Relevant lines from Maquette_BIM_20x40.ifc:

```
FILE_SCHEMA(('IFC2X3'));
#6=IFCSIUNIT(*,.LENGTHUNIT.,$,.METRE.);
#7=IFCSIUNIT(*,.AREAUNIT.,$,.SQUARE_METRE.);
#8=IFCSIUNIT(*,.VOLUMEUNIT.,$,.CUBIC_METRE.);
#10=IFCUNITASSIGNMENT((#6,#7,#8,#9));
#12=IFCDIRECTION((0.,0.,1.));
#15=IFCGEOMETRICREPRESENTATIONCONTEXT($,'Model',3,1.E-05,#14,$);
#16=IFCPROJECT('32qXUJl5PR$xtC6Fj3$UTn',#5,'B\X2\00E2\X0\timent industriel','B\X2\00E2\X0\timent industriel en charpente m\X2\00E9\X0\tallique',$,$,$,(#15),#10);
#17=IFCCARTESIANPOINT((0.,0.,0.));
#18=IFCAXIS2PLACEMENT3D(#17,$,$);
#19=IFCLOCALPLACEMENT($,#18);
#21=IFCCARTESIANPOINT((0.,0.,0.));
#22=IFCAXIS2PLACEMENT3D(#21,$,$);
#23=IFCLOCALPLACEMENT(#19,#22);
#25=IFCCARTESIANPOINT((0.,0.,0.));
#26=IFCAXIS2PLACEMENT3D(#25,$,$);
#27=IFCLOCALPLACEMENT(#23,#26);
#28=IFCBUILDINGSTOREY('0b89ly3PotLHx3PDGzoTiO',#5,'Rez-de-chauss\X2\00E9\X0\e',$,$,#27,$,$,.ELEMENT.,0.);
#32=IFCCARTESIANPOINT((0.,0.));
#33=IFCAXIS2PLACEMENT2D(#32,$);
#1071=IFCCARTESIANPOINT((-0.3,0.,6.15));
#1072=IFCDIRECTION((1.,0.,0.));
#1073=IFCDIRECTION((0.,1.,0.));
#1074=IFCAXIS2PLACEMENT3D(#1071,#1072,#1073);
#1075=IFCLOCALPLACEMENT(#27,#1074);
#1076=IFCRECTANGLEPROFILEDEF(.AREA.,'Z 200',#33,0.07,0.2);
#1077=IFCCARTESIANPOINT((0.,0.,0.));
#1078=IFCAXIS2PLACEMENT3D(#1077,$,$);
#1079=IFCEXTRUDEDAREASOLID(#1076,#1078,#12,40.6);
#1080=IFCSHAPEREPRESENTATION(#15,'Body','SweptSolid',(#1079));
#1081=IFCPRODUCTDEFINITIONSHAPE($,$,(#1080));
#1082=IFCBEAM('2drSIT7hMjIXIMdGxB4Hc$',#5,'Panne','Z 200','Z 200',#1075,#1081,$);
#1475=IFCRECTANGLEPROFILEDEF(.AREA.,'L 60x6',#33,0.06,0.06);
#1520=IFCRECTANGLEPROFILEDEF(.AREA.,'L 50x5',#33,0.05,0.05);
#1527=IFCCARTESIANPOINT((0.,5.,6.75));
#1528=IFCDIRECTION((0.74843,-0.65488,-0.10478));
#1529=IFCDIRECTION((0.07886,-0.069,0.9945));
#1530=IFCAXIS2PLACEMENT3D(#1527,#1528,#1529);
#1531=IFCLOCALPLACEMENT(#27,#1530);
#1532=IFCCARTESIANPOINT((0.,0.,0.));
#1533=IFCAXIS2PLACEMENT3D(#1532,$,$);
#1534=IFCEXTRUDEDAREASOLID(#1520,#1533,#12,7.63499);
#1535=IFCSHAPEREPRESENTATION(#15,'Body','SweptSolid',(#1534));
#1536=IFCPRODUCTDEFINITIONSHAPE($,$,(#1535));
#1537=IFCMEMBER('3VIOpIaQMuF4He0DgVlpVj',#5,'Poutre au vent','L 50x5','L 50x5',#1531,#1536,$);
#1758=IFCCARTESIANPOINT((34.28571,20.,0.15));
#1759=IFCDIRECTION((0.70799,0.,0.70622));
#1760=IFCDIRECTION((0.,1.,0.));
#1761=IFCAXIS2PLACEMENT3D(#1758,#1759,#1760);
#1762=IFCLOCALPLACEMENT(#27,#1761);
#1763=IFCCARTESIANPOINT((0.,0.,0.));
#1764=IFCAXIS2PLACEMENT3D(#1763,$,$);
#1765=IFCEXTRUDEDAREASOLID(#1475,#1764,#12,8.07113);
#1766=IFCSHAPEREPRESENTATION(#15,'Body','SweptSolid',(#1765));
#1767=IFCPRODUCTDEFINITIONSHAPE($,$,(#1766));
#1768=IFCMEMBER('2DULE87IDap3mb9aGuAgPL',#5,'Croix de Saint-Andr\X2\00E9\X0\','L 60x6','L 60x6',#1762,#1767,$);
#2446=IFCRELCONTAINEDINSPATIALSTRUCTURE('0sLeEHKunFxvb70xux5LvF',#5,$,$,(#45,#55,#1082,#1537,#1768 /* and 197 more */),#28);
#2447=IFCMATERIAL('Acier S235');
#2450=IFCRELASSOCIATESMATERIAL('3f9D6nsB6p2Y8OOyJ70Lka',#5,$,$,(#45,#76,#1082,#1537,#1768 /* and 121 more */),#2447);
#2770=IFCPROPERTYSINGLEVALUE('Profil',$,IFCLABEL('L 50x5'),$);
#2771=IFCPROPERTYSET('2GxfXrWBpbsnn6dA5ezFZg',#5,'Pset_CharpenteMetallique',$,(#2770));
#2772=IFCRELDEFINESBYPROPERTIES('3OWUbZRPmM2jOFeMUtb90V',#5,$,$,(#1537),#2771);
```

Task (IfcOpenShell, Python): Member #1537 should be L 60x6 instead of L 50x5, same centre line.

```python
import ifcopenshell
import ifcopenshell.api.pset
import ifcopenshell.util.element

model = ifcopenshell.open("Maquette_BIM_20x40.ifc")

member = model.by_guid("3VIOpIaQMuF4He0DgVlpVj")
source = next(p for p in model.by_type("IfcRectangleProfileDef") if p.ProfileName == "L 60x6")

body = next(r for r in member.Representation.Representations if r.RepresentationIdentifier == "Body")
solid = body.Items[0]
old_profile = solid.SweptArea

# Copy the section's sizes but keep this member's own profile position.
profile = ifcopenshell.util.element.copy(model, source)
profile.Position = old_profile.Position
solid.SweptArea = profile
if not model.get_total_inverses(old_profile):
    ifcopenshell.util.element.remove_deep2(model, old_profile)
member.Description = member.Description.replace("L 50x5", "L 60x6")
member.ObjectType = member.ObjectType.replace("L 50x5", "L 60x6")
pset = model.by_id(ifcopenshell.util.element.get_pset(member, "Pset_CharpenteMetallique", should_inherit=False)["id"])
ifcopenshell.api.pset.edit_pset(model, pset=pset, properties={"Profil": "L 60x6"})

print(solid.SweptArea)

model.write("Maquette_BIM_20x40_rev.ifc")
```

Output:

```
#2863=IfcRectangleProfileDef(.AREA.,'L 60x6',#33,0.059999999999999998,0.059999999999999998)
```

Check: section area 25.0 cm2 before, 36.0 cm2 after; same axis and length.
